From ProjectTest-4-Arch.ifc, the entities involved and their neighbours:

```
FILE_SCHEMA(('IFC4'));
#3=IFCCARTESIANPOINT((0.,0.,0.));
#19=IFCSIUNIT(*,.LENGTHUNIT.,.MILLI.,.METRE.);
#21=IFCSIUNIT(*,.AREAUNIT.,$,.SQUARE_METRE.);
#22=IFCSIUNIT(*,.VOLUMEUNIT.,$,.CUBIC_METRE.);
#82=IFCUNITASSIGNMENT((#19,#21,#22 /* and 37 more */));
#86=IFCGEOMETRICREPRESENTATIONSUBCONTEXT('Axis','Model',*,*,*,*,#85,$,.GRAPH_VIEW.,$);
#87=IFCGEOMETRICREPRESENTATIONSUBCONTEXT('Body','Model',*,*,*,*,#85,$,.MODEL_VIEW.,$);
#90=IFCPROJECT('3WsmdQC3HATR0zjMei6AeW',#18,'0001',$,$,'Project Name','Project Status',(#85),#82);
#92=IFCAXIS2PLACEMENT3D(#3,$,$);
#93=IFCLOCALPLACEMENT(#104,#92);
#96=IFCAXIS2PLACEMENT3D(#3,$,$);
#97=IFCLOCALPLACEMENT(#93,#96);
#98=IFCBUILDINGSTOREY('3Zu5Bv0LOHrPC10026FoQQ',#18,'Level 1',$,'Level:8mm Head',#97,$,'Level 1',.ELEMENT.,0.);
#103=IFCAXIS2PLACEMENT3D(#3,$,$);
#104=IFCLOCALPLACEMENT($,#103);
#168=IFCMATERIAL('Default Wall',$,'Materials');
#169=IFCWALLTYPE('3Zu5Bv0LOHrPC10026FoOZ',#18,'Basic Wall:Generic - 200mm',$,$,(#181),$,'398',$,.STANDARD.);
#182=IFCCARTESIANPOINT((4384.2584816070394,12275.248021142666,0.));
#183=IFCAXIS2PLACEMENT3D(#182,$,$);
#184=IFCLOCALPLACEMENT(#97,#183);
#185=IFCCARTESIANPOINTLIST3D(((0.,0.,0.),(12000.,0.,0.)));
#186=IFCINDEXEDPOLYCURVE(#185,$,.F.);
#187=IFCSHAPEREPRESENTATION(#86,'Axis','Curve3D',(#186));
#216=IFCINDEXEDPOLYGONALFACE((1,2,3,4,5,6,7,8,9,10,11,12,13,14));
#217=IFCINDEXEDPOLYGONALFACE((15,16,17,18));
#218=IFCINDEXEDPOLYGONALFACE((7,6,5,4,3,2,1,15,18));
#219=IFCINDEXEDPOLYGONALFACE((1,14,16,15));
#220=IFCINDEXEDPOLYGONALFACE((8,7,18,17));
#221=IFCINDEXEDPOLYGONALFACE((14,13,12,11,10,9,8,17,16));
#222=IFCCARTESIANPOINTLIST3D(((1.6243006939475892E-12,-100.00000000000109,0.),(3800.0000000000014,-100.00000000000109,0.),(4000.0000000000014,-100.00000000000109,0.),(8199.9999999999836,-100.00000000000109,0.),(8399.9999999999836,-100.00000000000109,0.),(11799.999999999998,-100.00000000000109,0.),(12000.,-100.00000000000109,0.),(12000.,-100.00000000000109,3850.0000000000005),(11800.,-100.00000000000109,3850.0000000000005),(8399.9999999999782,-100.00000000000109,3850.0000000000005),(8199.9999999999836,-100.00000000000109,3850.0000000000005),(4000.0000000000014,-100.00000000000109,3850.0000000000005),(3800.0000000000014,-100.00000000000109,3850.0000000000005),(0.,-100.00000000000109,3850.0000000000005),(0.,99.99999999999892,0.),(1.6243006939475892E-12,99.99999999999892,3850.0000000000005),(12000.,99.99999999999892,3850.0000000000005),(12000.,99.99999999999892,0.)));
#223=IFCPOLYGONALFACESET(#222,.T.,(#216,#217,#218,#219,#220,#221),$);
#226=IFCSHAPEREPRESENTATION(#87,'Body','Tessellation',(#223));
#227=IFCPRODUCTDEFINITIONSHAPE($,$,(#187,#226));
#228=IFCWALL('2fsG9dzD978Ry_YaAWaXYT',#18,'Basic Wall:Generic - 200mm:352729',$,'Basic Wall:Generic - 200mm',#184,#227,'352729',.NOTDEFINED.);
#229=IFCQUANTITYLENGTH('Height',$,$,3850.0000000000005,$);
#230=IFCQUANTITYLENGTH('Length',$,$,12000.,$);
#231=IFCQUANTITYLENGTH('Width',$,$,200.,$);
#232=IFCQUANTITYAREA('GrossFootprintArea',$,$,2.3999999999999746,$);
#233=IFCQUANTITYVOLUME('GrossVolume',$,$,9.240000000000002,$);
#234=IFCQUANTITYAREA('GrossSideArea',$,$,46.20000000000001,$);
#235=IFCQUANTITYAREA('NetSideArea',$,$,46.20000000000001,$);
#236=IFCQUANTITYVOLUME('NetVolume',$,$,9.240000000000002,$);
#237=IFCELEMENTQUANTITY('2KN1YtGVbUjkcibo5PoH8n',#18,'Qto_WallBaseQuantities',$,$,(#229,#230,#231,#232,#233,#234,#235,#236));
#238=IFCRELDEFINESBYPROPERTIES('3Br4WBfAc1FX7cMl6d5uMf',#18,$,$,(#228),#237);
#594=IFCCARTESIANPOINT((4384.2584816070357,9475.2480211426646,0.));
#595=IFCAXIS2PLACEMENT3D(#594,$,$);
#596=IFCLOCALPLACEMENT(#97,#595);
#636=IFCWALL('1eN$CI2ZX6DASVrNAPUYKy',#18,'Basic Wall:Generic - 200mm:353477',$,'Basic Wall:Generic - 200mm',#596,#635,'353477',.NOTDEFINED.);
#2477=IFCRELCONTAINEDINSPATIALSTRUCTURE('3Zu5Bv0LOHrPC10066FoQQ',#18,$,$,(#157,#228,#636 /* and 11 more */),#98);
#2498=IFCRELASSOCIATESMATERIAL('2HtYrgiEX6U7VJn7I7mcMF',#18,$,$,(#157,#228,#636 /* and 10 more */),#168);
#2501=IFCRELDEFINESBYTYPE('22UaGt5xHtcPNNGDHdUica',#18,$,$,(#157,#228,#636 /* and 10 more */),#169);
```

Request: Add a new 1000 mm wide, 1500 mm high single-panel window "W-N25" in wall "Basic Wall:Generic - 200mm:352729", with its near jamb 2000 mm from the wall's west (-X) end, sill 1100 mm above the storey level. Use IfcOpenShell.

```python
import numpy as np
import ifcopenshell
import ifcopenshell.api.feature
import ifcopenshell.api.geometry
import ifcopenshell.api.pset
import ifcopenshell.api.root
import ifcopenshell.api.spatial
import ifcopenshell.geom
import ifcopenshell.util.element
import ifcopenshell.util.placement
import ifcopenshell.util.representation
import ifcopenshell.util.shape
import ifcopenshell.util.unit

model = ifcopenshell.open("ProjectTest-4-Arch.ifc")
unit_scale = ifcopenshell.util.unit.calculate_unit_scale(model)
area_scale = ifcopenshell.util.unit.calculate_unit_scale(model, "AREAUNIT")
volume_scale = ifcopenshell.util.unit.calculate_unit_scale(model, "VOLUMEUNIT")
settings = ifcopenshell.geom.settings()


def volume(element):
    """Net volume in cubic metres, openings subtracted."""
    shape = ifcopenshell.geom.create_shape(settings, element)
    return ifcopenshell.util.shape.get_volume(shape.geometry)


wall = model.by_guid("2fsG9dzD978Ry_YaAWaXYT")
storey = ifcopenshell.util.element.get_container(wall, ifc_class="IfcBuildingStorey")
context = ifcopenshell.util.representation.get_context(model, "Model", "Body", "MODEL_VIEW")
before = volume(wall)

width, height, from_end, sill = 1, 1.5, 2, 1.1  # metres

# The wall runs along its own X axis, and the end named is its -X end.
wall_shape = ifcopenshell.geom.create_shape(settings, wall)
x, y, z = ifcopenshell.util.shape.get_vertices(wall_shape.geometry).T
start = x.min() + from_end
face, thickness = float(y.min()), float(y.max() - y.min())
wall_matrix = ifcopenshell.util.placement.get_local_placement(wall.ObjectPlacement)
level = ifcopenshell.util.placement.get_local_placement(storey.ObjectPlacement)[2, 3]


def in_wall(x, y):
    """Placement at x, y metres in the wall's axes, at sill height."""
    matrix = wall_matrix.copy()
    matrix[:, 3] = wall_matrix @ np.array([x / unit_scale, y / unit_scale, 0.0, 1.0])
    matrix[2, 3] = level + sill / unit_scale
    return matrix


# Opening: a box that overshoots both wall faces by 50 mm.
opening = ifcopenshell.api.root.create_entity(model, ifc_class="IfcOpeningElement", predefined_type="OPENING")
box = ifcopenshell.api.geometry.add_wall_representation(
    model, context=context, length=width, height=height, thickness=thickness + 0.1
)
ifcopenshell.api.geometry.assign_representation(model, product=opening, representation=box)
ifcopenshell.api.geometry.edit_object_placement(model, product=opening, matrix=in_wall(start, face - 0.05), is_si=False)
ifcopenshell.api.feature.add_feature(model, feature=opening, element=wall)

window = ifcopenshell.api.root.create_entity(model, ifc_class="IfcWindow", name="W-N25", predefined_type="WINDOW")
window.OverallWidth, window.OverallHeight = width / unit_scale, height / unit_scale
window.PartitioningType = "SINGLE_PANEL"
body = ifcopenshell.api.geometry.add_window_representation(
    model,
    context=context,
    overall_width=window.OverallWidth,
    overall_height=window.OverallHeight,
    partition_type="SINGLE_PANEL",
)
ifcopenshell.api.geometry.assign_representation(model, product=window, representation=body)
ifcopenshell.api.spatial.assign_container(model, products=[window], relating_structure=storey)
ifcopenshell.api.feature.add_filling(model, opening=opening, element=window)

# Centre the window in the wall's thickness.
ifcopenshell.api.geometry.edit_object_placement(model, product=window, matrix=in_wall(start, face), is_si=False)
window_shape = ifcopenshell.geom.create_shape(settings, window)
depth = ifcopenshell.util.shape.get_vertices(window_shape.geometry)[:, 1]
offset = face + thickness / 2 - (depth.min() + depth.max()) / 2
ifcopenshell.api.geometry.edit_object_placement(model, product=window, matrix=in_wall(start, offset), is_si=False)

after = volume(wall)

# Update the wall's stored quantities.
qto = model.by_id(ifcopenshell.util.element.get_pset(wall, "Qto_WallBaseQuantities", should_inherit=False)["id"])
ifcopenshell.api.pset.edit_qto(model, qto=qto, properties={
    "NetSideArea": after / thickness / area_scale,
    "NetVolume": after / volume_scale,
})

print(f"wall volume {before:.3f} -> {after:.3f} m3")

model.write("ProjectTest-4-Arch_rev.ifc")
```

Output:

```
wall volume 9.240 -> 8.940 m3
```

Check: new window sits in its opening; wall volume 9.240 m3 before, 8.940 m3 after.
